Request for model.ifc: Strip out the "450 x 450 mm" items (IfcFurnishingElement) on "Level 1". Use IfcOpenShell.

First a look at what the model holds.

```python
import ifcopenshell
import ifcopenshell.util.element

model = ifcopenshell.open("model.ifc")
print(model.schema)
storey = next(s for s in model.by_type("IfcBuildingStorey") if s.Name == "Level 1")
furniture = [e for e in ifcopenshell.util.element.get_decomposition(storey) if e.is_a("IfcFurnishingElement")]
seen = {}
for e in furniture:
    element_type = ifcopenshell.util.element.get_type(e)
    name = element_type.Name if element_type not in (None, e) else None
    seen[name] = seen.get(name, 0) + 1
for name, count in sorted(seen.items(), key=str):
    print(count, "x", name)
```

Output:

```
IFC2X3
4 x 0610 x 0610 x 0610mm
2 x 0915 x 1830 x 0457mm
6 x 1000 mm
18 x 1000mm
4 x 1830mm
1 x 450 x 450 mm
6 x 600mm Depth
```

```python
import ifcopenshell
import ifcopenshell.api.root
import ifcopenshell.util.element

model = ifcopenshell.open("model.ifc")

storey = next(s for s in model.by_type("IfcBuildingStorey") if s.Name == "Level 1")
furniture = [e for e in ifcopenshell.util.element.get_decomposition(storey) if e.is_a("IfcFurnishingElement")]
targets = [e for e in furniture if (t := ifcopenshell.util.element.get_type(e)) not in (None, e) and t.Name == "450 x 450 mm"]

for e in targets:
    ifcopenshell.api.root.remove_product(model, product=e)
print(len(targets), "removed")

model.write("model_updated.ifc")
```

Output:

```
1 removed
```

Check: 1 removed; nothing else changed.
